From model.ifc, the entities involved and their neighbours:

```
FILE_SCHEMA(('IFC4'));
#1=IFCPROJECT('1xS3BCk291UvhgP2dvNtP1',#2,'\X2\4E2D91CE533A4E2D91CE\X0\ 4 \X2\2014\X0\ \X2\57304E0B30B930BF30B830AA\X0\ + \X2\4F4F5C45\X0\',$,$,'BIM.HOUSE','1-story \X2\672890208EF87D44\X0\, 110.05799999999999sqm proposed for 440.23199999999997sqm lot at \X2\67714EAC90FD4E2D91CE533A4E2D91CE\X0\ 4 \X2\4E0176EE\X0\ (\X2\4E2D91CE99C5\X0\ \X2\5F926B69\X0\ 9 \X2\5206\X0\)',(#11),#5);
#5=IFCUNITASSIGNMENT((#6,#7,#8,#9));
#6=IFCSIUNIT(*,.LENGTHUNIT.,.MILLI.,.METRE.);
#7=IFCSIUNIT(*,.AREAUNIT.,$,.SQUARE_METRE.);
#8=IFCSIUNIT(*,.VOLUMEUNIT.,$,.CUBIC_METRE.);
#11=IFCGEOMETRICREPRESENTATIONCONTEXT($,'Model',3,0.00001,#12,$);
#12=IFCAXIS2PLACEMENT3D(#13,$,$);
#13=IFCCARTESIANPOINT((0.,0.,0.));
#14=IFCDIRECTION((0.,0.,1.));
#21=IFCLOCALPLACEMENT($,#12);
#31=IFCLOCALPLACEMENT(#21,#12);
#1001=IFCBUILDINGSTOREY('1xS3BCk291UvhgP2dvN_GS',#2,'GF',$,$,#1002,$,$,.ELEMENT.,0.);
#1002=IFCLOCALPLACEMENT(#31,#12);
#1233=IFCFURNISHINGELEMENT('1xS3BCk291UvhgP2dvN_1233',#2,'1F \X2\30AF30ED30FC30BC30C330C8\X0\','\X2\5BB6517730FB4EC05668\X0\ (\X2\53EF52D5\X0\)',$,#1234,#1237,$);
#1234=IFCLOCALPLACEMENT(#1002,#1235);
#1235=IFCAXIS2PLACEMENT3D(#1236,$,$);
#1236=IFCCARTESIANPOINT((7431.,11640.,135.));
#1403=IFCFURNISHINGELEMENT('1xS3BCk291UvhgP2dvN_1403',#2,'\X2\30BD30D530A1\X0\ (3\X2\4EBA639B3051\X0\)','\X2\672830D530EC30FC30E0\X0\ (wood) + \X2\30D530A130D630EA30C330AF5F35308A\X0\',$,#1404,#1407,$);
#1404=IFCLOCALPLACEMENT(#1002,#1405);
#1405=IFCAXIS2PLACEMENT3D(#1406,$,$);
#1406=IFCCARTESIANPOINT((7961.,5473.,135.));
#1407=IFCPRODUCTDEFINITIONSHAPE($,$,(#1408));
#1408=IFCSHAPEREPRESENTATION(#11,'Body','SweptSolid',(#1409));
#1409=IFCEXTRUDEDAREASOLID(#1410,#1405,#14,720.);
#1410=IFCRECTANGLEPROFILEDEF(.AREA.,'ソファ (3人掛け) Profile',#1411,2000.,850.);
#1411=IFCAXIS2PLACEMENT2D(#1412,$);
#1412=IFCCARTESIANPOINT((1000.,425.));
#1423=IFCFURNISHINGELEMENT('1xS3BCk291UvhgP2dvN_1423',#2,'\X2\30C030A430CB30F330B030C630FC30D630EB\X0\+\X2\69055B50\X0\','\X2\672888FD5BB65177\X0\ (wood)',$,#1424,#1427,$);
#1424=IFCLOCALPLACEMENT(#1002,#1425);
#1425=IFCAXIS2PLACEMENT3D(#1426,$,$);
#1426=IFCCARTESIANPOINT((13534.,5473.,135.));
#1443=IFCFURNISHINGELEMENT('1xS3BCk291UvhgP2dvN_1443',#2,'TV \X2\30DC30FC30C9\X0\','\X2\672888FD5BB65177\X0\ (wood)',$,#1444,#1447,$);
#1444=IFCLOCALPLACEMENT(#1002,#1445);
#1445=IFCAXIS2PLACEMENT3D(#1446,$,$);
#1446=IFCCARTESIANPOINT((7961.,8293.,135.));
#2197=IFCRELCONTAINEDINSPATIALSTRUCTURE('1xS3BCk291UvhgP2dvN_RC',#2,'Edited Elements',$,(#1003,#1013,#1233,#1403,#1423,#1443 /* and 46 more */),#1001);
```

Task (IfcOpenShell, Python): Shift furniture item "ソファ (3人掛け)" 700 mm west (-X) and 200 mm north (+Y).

```python
import ifcopenshell
import ifcopenshell.api.geometry
import ifcopenshell.util.placement
import ifcopenshell.util.unit

model = ifcopenshell.open("model.ifc")
unit_scale = ifcopenshell.util.unit.calculate_unit_scale(model)

item = model.by_guid("1xS3BCk291UvhgP2dvN_1403")
matrix = ifcopenshell.util.placement.get_local_placement(item.ObjectPlacement)
matrix[0, 3] -= 0.7 / unit_scale
matrix[1, 3] += 0.2 / unit_scale
ifcopenshell.api.geometry.edit_object_placement(model, product=item, matrix=matrix, is_si=False)

print(ifcopenshell.util.placement.get_local_placement(item.ObjectPlacement).round(3) + 0.0)

model.write("model-out.ifc")
```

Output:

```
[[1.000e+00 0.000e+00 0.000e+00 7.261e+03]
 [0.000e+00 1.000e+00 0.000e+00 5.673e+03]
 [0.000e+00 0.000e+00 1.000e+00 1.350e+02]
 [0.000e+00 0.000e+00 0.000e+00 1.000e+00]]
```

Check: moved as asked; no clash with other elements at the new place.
